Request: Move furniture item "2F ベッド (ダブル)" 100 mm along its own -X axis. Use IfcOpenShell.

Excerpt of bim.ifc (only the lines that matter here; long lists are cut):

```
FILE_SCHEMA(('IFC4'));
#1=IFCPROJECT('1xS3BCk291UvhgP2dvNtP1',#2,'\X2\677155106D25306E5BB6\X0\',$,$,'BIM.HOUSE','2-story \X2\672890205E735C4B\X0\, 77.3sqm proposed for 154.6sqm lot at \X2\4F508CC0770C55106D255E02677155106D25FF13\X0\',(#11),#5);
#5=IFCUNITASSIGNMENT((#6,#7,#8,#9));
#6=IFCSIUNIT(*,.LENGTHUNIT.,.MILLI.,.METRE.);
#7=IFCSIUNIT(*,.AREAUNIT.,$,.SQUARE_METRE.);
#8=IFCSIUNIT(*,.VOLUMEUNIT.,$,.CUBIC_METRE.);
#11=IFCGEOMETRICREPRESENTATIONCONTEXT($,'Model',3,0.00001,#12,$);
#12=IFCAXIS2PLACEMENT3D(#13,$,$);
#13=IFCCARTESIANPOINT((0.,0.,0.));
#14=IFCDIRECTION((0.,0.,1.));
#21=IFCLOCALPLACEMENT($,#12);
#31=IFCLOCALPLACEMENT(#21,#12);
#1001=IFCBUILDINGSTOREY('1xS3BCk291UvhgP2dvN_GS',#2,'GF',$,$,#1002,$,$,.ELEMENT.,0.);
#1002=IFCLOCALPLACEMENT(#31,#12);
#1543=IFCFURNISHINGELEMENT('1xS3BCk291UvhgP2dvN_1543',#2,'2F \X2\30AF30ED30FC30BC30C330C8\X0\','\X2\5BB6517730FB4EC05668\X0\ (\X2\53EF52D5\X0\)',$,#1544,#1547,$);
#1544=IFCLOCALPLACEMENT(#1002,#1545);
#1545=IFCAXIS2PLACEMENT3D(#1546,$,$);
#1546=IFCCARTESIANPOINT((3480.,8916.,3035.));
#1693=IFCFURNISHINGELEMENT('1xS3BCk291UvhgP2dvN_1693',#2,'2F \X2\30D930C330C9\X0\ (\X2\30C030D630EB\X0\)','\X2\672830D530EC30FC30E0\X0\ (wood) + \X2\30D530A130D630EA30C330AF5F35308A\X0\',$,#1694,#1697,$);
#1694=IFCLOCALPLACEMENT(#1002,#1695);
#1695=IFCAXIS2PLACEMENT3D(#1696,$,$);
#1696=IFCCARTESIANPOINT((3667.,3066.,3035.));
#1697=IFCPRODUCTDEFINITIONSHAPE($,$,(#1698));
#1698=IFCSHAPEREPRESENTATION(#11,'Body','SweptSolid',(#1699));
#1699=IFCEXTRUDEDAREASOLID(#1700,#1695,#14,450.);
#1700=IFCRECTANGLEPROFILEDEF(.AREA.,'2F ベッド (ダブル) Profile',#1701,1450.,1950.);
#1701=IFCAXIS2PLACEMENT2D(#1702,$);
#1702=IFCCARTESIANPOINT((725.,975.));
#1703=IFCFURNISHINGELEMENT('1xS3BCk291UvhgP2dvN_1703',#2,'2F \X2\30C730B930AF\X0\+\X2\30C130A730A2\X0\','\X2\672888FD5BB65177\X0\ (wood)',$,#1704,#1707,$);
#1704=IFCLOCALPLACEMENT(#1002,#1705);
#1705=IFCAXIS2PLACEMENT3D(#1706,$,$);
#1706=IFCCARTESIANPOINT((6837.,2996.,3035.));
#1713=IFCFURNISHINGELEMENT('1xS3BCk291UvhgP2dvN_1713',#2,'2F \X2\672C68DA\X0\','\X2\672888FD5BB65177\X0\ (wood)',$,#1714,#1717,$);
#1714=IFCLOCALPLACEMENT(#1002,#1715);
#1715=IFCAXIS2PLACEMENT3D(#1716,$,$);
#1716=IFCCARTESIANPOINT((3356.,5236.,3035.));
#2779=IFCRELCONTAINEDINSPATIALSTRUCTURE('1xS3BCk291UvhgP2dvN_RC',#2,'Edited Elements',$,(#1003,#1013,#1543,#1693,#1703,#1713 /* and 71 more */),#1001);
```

```python
import ifcopenshell
import ifcopenshell.api.geometry
import ifcopenshell.util.placement
import ifcopenshell.util.unit

model = ifcopenshell.open("bim.ifc")
unit_scale = ifcopenshell.util.unit.calculate_unit_scale(model)

item = model.by_guid("1xS3BCk291UvhgP2dvN_1693")
matrix = ifcopenshell.util.placement.get_local_placement(item.ObjectPlacement)
matrix[:3, 3] -= matrix[:3, 0] * 0.1 / unit_scale
ifcopenshell.api.geometry.edit_object_placement(model, product=item, matrix=matrix, is_si=False)

print(ifcopenshell.util.placement.get_local_placement(item.ObjectPlacement).round(3) + 0.0)

model.write("bim-out.ifc")
```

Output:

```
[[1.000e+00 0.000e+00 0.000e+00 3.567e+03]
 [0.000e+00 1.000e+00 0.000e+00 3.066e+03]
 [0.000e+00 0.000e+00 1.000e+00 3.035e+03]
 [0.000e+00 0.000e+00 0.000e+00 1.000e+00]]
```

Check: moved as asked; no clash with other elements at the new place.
